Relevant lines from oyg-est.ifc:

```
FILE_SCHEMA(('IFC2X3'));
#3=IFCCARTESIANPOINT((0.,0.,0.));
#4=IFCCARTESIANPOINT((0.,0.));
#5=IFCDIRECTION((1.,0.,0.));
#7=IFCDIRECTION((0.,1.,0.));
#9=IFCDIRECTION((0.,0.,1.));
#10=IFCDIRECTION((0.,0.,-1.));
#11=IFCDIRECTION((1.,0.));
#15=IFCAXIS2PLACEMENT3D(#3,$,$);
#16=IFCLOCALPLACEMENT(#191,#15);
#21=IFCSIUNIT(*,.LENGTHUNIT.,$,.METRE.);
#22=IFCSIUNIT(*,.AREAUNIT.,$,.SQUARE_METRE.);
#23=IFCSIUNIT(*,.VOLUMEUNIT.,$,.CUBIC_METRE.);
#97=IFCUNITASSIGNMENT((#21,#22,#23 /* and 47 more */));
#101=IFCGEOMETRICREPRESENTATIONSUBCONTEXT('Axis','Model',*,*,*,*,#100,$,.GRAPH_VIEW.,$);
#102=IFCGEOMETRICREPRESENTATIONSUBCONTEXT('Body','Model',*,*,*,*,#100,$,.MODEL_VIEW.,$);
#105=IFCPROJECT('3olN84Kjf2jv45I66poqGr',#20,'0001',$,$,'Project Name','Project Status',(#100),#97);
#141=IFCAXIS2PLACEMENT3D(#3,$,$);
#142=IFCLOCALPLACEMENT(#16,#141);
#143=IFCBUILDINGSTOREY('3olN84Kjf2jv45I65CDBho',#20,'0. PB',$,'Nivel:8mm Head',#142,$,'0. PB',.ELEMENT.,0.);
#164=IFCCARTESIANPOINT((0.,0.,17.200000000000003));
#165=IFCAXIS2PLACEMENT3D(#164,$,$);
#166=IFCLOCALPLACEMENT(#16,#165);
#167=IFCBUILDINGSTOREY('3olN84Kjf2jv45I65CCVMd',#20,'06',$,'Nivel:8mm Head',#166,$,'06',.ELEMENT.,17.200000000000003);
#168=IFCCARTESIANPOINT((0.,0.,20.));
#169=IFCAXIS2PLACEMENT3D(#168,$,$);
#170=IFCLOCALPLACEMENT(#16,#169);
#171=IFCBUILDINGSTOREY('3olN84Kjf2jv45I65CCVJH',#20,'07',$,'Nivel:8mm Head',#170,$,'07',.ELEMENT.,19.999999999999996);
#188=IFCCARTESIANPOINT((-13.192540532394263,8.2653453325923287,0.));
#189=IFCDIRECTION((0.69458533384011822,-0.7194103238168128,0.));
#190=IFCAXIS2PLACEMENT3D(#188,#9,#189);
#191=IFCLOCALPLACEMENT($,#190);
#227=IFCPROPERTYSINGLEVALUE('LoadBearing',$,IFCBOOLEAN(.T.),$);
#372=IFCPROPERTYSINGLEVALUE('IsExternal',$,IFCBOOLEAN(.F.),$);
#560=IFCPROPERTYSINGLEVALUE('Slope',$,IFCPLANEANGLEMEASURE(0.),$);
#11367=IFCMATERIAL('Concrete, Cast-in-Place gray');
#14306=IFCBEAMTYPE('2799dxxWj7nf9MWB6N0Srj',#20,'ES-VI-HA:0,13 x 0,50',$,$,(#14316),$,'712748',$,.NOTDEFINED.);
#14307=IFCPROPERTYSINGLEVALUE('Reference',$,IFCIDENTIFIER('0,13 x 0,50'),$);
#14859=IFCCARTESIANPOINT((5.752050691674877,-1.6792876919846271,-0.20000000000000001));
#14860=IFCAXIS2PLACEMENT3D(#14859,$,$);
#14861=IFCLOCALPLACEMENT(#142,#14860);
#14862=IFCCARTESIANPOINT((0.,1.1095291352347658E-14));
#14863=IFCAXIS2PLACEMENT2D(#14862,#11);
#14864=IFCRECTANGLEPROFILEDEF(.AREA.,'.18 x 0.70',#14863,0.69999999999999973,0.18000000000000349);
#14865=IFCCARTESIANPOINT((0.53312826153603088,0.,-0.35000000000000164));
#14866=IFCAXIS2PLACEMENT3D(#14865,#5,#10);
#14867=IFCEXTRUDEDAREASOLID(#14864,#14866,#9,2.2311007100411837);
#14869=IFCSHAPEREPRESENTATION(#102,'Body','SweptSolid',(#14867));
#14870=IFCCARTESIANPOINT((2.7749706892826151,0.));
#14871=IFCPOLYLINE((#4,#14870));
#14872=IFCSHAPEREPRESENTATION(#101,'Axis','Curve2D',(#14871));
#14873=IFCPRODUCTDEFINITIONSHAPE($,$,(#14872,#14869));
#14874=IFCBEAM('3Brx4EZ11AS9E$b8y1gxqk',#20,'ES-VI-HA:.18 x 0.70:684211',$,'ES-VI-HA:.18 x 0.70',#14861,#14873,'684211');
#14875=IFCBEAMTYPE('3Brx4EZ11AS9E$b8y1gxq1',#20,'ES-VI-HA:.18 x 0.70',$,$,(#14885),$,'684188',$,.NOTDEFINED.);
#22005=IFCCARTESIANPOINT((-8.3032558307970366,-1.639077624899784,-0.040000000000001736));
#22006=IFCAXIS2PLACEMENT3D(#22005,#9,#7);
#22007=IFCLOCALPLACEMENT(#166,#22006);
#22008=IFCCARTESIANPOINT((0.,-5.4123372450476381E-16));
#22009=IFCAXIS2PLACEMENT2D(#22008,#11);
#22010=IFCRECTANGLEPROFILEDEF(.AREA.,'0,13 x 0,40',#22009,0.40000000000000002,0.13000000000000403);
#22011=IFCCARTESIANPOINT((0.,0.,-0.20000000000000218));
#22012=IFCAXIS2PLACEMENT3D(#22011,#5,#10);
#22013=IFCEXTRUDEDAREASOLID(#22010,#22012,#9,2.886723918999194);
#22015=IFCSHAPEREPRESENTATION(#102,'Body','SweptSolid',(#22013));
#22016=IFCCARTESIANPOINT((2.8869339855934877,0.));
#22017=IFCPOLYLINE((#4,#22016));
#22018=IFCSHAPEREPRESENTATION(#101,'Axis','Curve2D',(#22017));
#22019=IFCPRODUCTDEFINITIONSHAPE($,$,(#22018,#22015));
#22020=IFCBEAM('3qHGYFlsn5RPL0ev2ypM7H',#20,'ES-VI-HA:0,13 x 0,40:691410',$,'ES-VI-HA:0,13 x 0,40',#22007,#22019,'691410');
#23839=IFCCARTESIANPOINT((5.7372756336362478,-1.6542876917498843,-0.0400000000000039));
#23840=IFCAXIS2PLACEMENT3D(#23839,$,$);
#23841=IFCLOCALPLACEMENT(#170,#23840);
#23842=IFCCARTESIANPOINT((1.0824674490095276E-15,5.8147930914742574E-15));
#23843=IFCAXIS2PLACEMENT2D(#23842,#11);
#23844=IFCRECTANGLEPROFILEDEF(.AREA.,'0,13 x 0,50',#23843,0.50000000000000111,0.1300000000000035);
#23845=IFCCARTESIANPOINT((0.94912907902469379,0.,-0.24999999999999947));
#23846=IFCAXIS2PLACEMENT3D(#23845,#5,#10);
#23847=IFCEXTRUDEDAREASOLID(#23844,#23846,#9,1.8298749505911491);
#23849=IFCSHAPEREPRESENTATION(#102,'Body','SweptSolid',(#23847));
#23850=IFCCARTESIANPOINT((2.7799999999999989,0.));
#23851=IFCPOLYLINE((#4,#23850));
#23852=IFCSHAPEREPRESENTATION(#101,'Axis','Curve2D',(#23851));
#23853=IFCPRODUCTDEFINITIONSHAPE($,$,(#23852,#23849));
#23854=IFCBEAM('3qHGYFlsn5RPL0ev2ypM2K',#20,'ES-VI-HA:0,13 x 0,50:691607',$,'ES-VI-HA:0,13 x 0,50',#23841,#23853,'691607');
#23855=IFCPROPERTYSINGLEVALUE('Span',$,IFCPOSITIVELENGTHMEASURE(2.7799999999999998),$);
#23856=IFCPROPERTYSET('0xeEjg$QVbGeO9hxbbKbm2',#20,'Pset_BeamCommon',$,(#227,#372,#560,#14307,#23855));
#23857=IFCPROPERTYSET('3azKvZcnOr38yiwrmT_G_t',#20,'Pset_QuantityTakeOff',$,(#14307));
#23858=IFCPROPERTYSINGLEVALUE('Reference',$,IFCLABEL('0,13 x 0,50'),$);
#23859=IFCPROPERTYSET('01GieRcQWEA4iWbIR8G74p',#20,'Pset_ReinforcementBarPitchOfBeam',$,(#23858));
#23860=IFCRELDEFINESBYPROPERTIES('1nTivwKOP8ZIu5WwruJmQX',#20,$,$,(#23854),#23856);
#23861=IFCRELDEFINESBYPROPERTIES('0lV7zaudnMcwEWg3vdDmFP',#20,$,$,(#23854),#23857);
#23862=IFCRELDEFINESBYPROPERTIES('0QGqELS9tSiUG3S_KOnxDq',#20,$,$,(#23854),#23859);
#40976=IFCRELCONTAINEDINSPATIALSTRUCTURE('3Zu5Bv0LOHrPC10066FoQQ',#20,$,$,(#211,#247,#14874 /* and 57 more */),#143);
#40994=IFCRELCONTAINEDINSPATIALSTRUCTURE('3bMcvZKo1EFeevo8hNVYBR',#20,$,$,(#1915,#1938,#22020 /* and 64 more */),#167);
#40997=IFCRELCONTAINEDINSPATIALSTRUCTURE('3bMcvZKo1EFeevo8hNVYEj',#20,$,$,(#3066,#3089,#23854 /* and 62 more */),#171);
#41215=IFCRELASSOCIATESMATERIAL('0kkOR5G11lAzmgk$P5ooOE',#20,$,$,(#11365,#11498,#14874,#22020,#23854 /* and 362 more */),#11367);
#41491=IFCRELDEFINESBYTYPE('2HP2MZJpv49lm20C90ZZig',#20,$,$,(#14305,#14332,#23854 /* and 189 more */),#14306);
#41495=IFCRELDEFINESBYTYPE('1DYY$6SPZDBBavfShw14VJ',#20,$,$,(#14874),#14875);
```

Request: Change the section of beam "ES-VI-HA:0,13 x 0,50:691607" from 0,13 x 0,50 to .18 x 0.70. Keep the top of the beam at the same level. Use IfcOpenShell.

```python
import ifcopenshell
import ifcopenshell.api.pset
import ifcopenshell.api.type
import ifcopenshell.util.element
import ifcopenshell.util.representation

model = ifcopenshell.open("oyg-est.ifc")

member = model.by_guid("3qHGYFlsn5RPL0ev2ypM2K")
source = next(p for p in model.by_type("IfcRectangleProfileDef") if p.ProfileName == ".18 x 0.70")

body = ifcopenshell.util.representation.get_representation(member, "Model", "Body")
solid = body.Items[0]
old_profile = solid.SweptArea

# Copy the section's sizes but keep this member's own profile position.
profile = ifcopenshell.util.element.copy(model, source)
# Profiles are centred, so shift by half the change in depth to hold the top.
shift = (old_profile.XDim - profile.XDim) / 2
x, y = old_profile.Position.Location.Coordinates
up = (-1.0, 0.0)  # upwards, in the solid's own plane
location = model.createIfcCartesianPoint((x + up[0] * shift, y + up[1] * shift))
profile.Position = model.createIfcAxis2Placement2D(location, old_profile.Position.RefDirection)
solid.SweptArea = profile
if not model.get_total_inverses(old_profile):
    ifcopenshell.util.element.remove_deep2(model, old_profile)

new_type = model.by_id(14875)
ifcopenshell.api.type.assign_type(
    model, related_objects=[member], relating_type=new_type, should_map_representations=False
)
member.Name = member.Name.replace("0,13 x 0,50", ".18 x 0.70")
member.ObjectType = "ES-VI-HA:.18 x 0.70"
pset = model.by_id(ifcopenshell.util.element.get_pset(member, "Pset_BeamCommon", should_inherit=False)["id"])
ifcopenshell.api.pset.edit_pset(model, pset=pset, properties={"Reference": ".18 x 0.70"})
pset = model.by_id(ifcopenshell.util.element.get_pset(member, "Pset_QuantityTakeOff", should_inherit=False)["id"])
ifcopenshell.api.pset.edit_pset(model, pset=pset, properties={"Reference": ".18 x 0.70"})
pset = model.by_id(ifcopenshell.util.element.get_pset(member, "Pset_ReinforcementBarPitchOfBeam", should_inherit=False)["id"])
ifcopenshell.api.pset.edit_pset(model, pset=pset, properties={"Reference": ".18 x 0.70"})

print(solid.SweptArea)

model.write("oyg-est_v2.ifc")
```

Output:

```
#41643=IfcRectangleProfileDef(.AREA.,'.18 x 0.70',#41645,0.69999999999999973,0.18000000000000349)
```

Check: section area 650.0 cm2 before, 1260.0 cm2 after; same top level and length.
